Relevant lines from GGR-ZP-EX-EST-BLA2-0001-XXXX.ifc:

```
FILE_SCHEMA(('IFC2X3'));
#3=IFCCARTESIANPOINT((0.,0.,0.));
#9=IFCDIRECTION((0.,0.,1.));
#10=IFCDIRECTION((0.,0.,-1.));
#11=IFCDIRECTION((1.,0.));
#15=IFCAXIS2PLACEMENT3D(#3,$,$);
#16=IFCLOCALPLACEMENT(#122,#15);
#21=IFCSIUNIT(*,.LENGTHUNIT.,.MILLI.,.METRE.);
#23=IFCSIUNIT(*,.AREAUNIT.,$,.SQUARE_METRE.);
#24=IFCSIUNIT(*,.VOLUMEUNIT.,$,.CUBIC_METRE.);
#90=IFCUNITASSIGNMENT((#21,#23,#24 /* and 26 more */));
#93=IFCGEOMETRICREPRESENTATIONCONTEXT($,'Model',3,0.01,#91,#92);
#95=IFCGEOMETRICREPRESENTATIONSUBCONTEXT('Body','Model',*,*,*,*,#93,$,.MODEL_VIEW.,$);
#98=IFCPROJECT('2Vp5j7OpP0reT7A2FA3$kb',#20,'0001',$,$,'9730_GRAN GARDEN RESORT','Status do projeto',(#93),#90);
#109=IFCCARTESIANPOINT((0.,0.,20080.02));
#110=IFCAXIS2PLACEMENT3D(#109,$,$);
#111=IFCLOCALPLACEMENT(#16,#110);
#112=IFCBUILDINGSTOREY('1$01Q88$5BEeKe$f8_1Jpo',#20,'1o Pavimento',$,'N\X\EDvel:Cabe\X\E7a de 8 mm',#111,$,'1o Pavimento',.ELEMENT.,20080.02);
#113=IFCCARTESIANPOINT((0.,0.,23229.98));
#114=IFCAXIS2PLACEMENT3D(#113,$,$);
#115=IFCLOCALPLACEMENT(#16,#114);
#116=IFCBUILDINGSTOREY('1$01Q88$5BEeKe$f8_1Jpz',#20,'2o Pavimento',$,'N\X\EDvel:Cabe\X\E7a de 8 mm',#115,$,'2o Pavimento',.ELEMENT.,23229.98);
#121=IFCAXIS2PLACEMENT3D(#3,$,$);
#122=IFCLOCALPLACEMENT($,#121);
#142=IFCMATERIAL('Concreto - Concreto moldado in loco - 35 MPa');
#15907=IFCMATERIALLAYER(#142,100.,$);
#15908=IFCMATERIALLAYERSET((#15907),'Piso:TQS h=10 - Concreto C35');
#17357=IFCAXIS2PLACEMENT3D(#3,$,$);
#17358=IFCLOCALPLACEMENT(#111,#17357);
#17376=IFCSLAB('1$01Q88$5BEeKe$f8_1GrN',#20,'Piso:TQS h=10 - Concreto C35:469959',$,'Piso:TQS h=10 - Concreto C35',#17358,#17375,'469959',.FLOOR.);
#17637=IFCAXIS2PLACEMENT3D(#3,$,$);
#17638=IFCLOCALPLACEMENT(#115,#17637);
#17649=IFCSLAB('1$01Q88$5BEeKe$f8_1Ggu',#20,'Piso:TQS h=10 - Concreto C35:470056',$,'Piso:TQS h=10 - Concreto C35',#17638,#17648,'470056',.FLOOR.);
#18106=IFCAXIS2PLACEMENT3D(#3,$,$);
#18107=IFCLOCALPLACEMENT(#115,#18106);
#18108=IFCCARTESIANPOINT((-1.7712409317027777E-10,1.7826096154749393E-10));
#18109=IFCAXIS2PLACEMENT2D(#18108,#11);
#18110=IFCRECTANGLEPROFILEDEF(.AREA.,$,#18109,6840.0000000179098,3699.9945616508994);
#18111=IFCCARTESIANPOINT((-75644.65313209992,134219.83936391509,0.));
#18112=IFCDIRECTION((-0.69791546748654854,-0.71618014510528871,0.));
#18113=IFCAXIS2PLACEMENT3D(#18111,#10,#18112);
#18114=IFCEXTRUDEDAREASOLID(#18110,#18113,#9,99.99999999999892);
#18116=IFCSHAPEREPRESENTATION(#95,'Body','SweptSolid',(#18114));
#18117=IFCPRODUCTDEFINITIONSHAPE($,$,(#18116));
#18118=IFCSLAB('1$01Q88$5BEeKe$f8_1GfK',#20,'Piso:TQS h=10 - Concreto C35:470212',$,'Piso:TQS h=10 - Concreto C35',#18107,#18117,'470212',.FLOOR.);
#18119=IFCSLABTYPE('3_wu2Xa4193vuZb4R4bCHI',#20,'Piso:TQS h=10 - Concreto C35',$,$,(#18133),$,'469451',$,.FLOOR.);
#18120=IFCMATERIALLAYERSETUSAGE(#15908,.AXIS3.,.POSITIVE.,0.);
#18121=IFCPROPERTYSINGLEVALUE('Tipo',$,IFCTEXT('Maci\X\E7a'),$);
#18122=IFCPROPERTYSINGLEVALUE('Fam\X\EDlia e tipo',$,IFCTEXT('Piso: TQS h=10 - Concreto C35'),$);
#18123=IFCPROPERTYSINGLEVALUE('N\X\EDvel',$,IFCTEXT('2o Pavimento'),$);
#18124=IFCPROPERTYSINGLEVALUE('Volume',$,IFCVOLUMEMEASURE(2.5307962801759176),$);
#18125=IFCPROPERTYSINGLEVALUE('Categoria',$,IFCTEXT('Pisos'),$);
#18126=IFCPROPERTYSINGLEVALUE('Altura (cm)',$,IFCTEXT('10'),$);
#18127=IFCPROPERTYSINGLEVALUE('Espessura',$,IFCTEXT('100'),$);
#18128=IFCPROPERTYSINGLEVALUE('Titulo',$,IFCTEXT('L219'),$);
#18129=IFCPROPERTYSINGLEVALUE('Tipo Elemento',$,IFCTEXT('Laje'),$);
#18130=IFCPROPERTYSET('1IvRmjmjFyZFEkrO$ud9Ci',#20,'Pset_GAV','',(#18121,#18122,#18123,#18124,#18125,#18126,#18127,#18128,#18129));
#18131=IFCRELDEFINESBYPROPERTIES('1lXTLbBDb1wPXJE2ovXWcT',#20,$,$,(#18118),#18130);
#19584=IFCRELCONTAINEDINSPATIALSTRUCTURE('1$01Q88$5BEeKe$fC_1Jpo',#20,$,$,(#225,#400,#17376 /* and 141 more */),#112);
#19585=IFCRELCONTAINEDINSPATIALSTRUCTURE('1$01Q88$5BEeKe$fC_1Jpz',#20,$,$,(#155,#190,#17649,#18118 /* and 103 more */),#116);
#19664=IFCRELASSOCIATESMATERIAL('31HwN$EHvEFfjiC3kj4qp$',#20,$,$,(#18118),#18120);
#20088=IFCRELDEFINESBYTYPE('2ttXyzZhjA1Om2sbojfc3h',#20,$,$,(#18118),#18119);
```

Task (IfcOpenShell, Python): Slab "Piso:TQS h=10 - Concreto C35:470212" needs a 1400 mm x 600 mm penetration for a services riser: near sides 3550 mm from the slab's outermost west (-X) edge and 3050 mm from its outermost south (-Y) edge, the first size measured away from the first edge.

```python
import numpy as np
import ifcopenshell
import ifcopenshell.api.feature
import ifcopenshell.api.geometry
import ifcopenshell.api.pset
import ifcopenshell.api.root
import ifcopenshell.geom
import ifcopenshell.util.element
import ifcopenshell.util.placement
import ifcopenshell.util.representation
import ifcopenshell.util.shape
import ifcopenshell.util.unit

model = ifcopenshell.open("GGR-ZP-EX-EST-BLA2-0001-XXXX.ifc")
unit_scale = ifcopenshell.util.unit.calculate_unit_scale(model)
volume_scale = ifcopenshell.util.unit.calculate_unit_scale(model, "VOLUMEUNIT")
settings = ifcopenshell.geom.settings()


def volume(element):
    """Net volume in cubic metres, openings subtracted."""
    shape = ifcopenshell.geom.create_shape(settings, element)
    return ifcopenshell.util.shape.get_volume(shape.geometry)


slab = model.by_guid("1$01Q88$5BEeKe$f8_1GfK")
before = volume(slab)

# Extent in the slab's own axes, in metres. The edges named are its -X and -Y sides.
slab_shape = ifcopenshell.geom.create_shape(settings, slab)
vertices = ifcopenshell.util.shape.get_vertices(slab_shape.geometry)
x_min, y_min, bottom = vertices.min(axis=0)
top = vertices[:, 2].max()

opening = ifcopenshell.api.root.create_entity(model, ifc_class="IfcOpeningElement", name="Services riser opening")
context = ifcopenshell.util.representation.get_context(model, "Model", "Body", "MODEL_VIEW")
width, depth = 1.4, 0.6
outline = [(0.0, 0.0), (width, 0.0), (width, depth), (0.0, depth), (0.0, 0.0)]
# Overshoot both faces by 50 mm so the cut is clean.
shape = ifcopenshell.api.geometry.add_slab_representation(
    model, context=context, depth=top - bottom + 0.1, polyline=outline
)
ifcopenshell.api.geometry.assign_representation(model, product=opening, representation=shape)

matrix = ifcopenshell.util.placement.get_local_placement(slab.ObjectPlacement)
matrix[:, 3] = matrix @ np.append(np.array([x_min + 3.55, y_min + 3.05, bottom - 0.05]) / unit_scale, 1.0)
ifcopenshell.api.geometry.edit_object_placement(model, product=opening, matrix=matrix, is_si=False)
ifcopenshell.api.feature.add_feature(model, feature=opening, element=slab)

after = volume(slab)

# Update the slab's stored quantities.
pset = model.by_id(ifcopenshell.util.element.get_pset(slab, "Pset_GAV", should_inherit=False)["id"])
ifcopenshell.api.pset.edit_pset(model, pset=pset, properties={
    "Volume": model.create_entity("IfcVolumeMeasure", after / volume_scale),
})

print(f"slab volume {before:.3f} -> {after:.3f} m3")

model.write("GGR-ZP-EX-EST-BLA2-0001-XXXX_v2.ifc")
```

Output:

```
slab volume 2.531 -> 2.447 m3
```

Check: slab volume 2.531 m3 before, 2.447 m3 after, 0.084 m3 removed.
